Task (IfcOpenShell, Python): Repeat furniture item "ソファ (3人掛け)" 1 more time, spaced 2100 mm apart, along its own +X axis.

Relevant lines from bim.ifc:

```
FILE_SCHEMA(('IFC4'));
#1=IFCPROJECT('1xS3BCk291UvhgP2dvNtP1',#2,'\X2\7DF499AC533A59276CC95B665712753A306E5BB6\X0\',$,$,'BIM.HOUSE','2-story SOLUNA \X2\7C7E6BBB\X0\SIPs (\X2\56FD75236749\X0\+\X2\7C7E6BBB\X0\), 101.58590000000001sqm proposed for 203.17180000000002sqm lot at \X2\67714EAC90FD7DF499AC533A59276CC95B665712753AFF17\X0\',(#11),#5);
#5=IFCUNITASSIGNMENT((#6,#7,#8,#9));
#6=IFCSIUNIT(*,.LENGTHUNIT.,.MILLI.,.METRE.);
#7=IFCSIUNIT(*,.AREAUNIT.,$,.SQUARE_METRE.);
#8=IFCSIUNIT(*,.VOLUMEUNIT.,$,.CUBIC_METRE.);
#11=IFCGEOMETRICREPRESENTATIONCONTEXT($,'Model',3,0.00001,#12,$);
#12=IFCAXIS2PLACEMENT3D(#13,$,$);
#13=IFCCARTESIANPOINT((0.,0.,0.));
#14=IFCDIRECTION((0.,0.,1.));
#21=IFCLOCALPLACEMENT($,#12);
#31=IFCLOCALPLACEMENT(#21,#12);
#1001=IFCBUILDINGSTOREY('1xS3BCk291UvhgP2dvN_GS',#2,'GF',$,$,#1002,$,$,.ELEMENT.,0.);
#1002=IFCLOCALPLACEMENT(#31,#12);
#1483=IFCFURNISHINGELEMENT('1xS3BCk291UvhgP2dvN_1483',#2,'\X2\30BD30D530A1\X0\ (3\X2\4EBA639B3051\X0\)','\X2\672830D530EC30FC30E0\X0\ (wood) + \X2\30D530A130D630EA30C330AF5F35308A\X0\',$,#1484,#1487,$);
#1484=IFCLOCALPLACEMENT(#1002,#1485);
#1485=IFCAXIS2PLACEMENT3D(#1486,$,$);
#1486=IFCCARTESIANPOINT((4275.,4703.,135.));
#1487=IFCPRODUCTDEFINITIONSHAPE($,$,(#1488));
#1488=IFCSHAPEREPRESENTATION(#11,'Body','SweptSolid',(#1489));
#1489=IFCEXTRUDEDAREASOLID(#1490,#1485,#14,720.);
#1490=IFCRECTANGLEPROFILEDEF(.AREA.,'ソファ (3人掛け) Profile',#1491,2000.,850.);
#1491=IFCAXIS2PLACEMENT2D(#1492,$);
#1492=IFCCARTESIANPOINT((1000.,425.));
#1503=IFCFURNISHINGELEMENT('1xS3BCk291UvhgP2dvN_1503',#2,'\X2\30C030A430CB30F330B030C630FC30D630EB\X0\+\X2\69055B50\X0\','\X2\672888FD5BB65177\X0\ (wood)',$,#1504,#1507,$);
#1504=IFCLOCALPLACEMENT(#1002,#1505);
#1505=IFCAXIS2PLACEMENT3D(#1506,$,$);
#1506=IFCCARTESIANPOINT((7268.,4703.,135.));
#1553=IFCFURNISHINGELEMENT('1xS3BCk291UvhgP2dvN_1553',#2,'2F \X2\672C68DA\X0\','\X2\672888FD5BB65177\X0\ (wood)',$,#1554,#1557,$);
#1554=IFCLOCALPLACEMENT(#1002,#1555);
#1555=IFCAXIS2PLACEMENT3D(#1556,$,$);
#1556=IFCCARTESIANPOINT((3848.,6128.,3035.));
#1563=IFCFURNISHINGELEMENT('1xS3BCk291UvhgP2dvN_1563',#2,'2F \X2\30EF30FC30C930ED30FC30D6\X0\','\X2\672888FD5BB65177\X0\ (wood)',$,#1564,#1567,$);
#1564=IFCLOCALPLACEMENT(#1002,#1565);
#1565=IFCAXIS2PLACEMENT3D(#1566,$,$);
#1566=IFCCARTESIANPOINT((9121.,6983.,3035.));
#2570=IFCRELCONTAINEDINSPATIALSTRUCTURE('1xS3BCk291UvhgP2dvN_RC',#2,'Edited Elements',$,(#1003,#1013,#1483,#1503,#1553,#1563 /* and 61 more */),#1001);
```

```python
import ifcopenshell
import ifcopenshell.api.geometry
import ifcopenshell.api.root
import ifcopenshell.util.element
import ifcopenshell.util.placement
import ifcopenshell.util.unit

model = ifcopenshell.open("bim.ifc")
unit_scale = ifcopenshell.util.unit.calculate_unit_scale(model)


def reuse_history(source, copy):
    """copy_class also copies each property set's owner history, people and application; keep the originals."""
    for rel in copy.IsDefinedBy:
        if rel.is_a("IfcRelDefinesByProperties") and (history := rel.RelatingPropertyDefinition.OwnerHistory):
            rel.RelatingPropertyDefinition.OwnerHistory = source.OwnerHistory
            ifcopenshell.util.element.remove_deep2(model, history)


source = model.by_guid("1xS3BCk291UvhgP2dvN_1483")
base = ifcopenshell.util.placement.get_local_placement(source.ObjectPlacement)
step = base[:3, 0] * 2.1 / unit_scale

for i in range(1, 2):
    copy = ifcopenshell.api.root.copy_class(model, product=source)
    copy.Representation = ifcopenshell.util.element.copy_deep(
        model, source.Representation, exclude=["IfcGeometricRepresentationContext", "IfcRepresentationMap"]
    )
    reuse_history(source, copy)
    matrix = base.copy()
    matrix[:3, 3] += i * step
    print("added at", matrix[:3, 3].round(3) + 0.0)
    ifcopenshell.api.geometry.edit_object_placement(model, product=copy, matrix=matrix, is_si=False)

model.write("bim_edited.ifc")
```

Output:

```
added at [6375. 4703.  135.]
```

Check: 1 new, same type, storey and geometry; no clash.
